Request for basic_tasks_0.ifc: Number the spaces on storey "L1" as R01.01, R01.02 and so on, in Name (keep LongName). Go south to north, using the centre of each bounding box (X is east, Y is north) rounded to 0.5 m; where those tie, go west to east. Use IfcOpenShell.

First a look at what the model holds.

```python
import ifcopenshell
import ifcopenshell.util.element
import ifcopenshell.util.placement

model = ifcopenshell.open("basic_tasks_0.ifc")
print(model.schema)
storey = next(s for s in model.by_type("IfcBuildingStorey") if s.Name == "L1")
spaces = [e for e in ifcopenshell.util.element.get_decomposition(storey) if e.is_a("IfcSpace")]
for e in sorted(spaces, key=lambda e: e.id()):
    origin = ifcopenshell.util.placement.get_local_placement(e.ObjectPlacement)[:3, 3]
    print(e.id(), e.Name, e.LongName, origin.round(2) + 0.0, sep=" | ")
```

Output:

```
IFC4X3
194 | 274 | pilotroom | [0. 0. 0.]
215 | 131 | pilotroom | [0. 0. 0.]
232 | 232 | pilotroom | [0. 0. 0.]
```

```python
import ifcopenshell
import ifcopenshell.geom
import ifcopenshell.util.element
import ifcopenshell.util.shape

model = ifcopenshell.open("basic_tasks_0.ifc")
settings = ifcopenshell.geom.settings()
settings.set("use-world-coords", True)


def centre(element):
    shape = ifcopenshell.geom.create_shape(settings, element)
    return ifcopenshell.util.shape.get_bbox_centroid(shape.geometry)


storey = next(s for s in model.by_type("IfcBuildingStorey") if s.Name == "L1")
spaces = [e for e in ifcopenshell.util.element.get_decomposition(storey) if e.is_a("IfcSpace")]

# Insertion points can sit at a corner or the storey origin, so sort by the geometry (in metres).
centres = {e: centre(e) for e in spaces}
spaces.sort(key=lambda e: (round(centres[e][1] / 0.5), centres[e][0]))

for i, e in enumerate(spaces, start=1):
    number = f"R01.{i:02d}"
    e.Name = number
    print(e.id(), number)

model.write("basic_tasks_0_updated.ifc")
```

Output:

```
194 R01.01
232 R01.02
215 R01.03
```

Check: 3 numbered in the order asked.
